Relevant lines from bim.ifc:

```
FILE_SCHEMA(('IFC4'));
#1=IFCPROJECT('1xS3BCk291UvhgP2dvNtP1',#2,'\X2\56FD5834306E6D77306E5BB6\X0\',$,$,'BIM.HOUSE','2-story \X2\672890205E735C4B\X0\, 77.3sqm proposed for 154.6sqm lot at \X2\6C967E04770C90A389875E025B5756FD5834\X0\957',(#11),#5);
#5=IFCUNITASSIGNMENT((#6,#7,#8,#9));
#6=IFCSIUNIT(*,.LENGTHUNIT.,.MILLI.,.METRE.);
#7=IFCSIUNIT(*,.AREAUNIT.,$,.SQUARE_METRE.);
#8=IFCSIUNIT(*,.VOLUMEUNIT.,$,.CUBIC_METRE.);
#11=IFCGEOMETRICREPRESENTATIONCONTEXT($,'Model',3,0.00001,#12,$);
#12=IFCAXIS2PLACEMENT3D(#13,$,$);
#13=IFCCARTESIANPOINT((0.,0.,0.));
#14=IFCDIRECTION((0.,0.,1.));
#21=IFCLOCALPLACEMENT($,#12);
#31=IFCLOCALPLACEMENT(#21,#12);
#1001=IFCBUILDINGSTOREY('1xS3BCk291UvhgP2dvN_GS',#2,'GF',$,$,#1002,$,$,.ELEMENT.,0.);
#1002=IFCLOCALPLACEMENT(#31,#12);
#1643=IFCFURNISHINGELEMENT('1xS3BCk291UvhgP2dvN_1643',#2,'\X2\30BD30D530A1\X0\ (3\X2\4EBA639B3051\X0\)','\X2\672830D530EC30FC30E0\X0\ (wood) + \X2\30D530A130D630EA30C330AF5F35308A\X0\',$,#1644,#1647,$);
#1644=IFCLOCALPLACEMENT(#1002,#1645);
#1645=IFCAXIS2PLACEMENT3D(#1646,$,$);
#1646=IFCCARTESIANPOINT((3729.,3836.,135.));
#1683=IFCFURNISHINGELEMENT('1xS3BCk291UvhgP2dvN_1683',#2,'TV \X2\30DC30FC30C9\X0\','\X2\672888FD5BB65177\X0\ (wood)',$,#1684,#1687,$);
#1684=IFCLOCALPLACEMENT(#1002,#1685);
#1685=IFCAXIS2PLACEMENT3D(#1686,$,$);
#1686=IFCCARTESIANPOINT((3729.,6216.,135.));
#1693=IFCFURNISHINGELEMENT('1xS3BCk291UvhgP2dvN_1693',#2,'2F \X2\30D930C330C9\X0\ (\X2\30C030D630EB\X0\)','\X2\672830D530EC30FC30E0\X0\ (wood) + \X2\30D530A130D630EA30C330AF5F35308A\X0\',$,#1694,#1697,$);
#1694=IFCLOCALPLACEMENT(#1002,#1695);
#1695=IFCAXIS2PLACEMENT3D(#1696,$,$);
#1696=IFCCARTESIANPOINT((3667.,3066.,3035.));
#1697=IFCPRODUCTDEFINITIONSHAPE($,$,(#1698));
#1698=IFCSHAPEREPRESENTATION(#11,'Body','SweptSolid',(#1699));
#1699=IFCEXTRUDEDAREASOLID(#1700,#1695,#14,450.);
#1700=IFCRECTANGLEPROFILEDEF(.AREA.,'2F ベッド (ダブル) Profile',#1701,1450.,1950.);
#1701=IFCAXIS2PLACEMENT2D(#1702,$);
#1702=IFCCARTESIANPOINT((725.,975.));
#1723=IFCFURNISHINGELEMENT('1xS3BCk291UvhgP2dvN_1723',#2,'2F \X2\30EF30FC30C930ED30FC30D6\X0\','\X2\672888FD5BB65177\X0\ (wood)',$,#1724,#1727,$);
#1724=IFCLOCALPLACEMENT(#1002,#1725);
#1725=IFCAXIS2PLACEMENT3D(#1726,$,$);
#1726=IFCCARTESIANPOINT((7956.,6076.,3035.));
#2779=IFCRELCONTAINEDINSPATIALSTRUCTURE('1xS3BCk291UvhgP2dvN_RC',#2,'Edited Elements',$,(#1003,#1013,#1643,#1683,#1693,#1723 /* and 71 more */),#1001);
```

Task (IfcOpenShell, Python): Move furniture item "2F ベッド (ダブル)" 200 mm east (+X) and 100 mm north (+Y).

```python
import ifcopenshell
import ifcopenshell.api.geometry
import ifcopenshell.util.placement
import ifcopenshell.util.unit

model = ifcopenshell.open("bim.ifc")
unit_scale = ifcopenshell.util.unit.calculate_unit_scale(model)

item = model.by_id(1693)
matrix = ifcopenshell.util.placement.get_local_placement(item.ObjectPlacement)
matrix[0, 3] += 0.2 / unit_scale
matrix[1, 3] += 0.1 / unit_scale
ifcopenshell.api.geometry.edit_object_placement(model, product=item, matrix=matrix, is_si=False)

print(ifcopenshell.util.placement.get_local_placement(item.ObjectPlacement).round(3) + 0.0)

model.write("bim_rev.ifc")
```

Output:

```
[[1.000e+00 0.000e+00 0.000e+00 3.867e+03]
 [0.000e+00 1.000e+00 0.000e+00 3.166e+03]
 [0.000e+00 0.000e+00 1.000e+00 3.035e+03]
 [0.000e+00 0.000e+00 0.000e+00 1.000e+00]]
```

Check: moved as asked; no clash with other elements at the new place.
